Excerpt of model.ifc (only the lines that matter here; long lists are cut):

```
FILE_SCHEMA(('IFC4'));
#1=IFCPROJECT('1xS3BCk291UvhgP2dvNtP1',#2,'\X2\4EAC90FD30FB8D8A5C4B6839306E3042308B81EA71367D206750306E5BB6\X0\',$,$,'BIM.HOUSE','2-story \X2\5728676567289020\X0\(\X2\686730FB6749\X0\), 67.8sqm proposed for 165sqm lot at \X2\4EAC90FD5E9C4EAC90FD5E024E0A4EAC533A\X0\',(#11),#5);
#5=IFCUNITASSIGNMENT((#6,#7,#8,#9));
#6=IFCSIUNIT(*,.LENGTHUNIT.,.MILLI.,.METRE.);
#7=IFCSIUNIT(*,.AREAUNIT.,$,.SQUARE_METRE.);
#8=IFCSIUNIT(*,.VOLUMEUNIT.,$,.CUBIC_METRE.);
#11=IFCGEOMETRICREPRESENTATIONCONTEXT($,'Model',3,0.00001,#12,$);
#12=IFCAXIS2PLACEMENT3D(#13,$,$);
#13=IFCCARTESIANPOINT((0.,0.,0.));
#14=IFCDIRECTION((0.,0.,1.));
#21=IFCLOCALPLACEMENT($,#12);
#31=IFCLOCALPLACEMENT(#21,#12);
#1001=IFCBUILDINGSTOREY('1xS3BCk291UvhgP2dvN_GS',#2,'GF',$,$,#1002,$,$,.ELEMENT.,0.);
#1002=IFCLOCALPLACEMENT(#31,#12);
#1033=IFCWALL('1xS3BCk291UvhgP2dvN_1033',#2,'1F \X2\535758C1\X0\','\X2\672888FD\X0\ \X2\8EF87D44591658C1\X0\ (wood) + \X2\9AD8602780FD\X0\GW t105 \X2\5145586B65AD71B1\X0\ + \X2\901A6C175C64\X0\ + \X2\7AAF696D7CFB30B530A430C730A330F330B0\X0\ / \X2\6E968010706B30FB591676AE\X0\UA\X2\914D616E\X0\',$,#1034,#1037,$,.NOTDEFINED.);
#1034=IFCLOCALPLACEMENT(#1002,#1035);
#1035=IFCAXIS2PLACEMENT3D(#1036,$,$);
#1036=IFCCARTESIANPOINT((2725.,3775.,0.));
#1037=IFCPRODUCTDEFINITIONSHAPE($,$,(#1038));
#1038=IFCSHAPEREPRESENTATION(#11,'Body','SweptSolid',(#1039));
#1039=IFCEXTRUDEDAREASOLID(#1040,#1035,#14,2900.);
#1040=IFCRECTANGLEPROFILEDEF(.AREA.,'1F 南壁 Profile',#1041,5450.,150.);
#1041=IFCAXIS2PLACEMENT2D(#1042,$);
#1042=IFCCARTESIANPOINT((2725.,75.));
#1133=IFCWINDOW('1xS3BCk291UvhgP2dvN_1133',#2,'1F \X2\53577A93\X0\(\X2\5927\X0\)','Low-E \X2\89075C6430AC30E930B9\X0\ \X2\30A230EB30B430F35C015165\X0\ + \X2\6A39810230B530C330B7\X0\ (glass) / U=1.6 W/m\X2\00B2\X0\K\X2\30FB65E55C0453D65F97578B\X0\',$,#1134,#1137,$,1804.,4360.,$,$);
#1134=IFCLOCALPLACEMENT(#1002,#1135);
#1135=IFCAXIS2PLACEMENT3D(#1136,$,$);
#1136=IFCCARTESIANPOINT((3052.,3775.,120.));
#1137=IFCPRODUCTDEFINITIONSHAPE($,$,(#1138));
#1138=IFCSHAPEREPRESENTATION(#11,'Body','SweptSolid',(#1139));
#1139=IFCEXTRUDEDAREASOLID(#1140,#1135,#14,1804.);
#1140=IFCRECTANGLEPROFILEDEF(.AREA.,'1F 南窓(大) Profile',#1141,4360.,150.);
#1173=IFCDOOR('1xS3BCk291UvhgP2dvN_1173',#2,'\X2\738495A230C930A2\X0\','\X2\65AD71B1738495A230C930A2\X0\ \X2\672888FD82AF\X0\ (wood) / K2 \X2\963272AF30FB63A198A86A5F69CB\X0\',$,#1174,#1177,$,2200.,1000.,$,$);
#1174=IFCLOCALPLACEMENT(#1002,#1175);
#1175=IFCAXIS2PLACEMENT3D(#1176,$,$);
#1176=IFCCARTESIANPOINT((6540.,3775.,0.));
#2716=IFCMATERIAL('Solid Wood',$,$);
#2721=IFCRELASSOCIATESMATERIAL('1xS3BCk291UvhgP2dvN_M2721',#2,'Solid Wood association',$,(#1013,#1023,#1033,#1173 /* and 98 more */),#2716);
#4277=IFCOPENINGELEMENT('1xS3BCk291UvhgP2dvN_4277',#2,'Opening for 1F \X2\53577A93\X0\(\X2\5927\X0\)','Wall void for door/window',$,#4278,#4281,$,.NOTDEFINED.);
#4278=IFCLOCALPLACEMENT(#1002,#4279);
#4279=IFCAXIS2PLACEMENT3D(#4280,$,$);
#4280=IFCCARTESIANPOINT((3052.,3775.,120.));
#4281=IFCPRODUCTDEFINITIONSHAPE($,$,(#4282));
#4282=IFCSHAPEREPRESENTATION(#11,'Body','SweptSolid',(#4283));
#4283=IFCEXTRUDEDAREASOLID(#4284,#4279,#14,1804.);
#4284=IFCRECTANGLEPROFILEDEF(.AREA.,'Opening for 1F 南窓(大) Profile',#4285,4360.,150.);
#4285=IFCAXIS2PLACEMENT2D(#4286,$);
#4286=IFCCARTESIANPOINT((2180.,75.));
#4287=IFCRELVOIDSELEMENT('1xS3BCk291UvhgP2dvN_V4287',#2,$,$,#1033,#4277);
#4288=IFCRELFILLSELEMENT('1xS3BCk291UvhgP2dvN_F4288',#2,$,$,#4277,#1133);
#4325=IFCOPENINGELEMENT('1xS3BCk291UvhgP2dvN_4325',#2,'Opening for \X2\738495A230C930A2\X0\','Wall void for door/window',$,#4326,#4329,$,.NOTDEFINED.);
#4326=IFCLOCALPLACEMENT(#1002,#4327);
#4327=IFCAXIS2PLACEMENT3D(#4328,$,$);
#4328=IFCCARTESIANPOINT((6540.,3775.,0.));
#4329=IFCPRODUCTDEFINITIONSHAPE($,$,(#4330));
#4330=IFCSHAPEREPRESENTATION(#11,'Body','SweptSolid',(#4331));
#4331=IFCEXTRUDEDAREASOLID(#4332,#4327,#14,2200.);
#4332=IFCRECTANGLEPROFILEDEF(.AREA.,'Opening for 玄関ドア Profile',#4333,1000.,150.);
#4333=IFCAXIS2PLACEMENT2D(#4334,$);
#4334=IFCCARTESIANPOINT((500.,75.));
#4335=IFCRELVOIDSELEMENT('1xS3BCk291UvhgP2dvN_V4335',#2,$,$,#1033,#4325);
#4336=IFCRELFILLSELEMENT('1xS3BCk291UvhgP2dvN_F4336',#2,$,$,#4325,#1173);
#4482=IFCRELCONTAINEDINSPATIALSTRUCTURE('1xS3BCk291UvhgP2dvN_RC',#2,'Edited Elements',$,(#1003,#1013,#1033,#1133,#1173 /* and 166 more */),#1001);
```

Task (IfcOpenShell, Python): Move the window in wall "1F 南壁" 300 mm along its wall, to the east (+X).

```python
import ifcopenshell
import ifcopenshell.api.geometry
import ifcopenshell.util.placement

model = ifcopenshell.open("model.ifc")

window = model.by_guid("1xS3BCk291UvhgP2dvN_1133")
opening = window.FillsVoids[0].RelatingOpeningElement
wall = opening.VoidsElements[0].RelatingBuildingElement

wall_matrix = ifcopenshell.util.placement.get_local_placement(wall.ObjectPlacement)
shift = wall_matrix[:3, 0] * 300.0
before = ifcopenshell.util.placement.get_local_placement(window.ObjectPlacement)[:3, 3].copy()

# The window is not placed relative to its opening, so move both.
for product in (opening, window):
    matrix = ifcopenshell.util.placement.get_local_placement(product.ObjectPlacement)
    matrix[:3, 3] += shift
    ifcopenshell.api.geometry.edit_object_placement(model, product=product, matrix=matrix, is_si=False)

after = ifcopenshell.util.placement.get_local_placement(window.ObjectPlacement)[:3, 3]
print("window moved by", (after - before).round(3) + 0.0)

model.write("model_v2.ifc")
```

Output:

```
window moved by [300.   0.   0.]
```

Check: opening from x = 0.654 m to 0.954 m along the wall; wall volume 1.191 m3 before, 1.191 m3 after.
